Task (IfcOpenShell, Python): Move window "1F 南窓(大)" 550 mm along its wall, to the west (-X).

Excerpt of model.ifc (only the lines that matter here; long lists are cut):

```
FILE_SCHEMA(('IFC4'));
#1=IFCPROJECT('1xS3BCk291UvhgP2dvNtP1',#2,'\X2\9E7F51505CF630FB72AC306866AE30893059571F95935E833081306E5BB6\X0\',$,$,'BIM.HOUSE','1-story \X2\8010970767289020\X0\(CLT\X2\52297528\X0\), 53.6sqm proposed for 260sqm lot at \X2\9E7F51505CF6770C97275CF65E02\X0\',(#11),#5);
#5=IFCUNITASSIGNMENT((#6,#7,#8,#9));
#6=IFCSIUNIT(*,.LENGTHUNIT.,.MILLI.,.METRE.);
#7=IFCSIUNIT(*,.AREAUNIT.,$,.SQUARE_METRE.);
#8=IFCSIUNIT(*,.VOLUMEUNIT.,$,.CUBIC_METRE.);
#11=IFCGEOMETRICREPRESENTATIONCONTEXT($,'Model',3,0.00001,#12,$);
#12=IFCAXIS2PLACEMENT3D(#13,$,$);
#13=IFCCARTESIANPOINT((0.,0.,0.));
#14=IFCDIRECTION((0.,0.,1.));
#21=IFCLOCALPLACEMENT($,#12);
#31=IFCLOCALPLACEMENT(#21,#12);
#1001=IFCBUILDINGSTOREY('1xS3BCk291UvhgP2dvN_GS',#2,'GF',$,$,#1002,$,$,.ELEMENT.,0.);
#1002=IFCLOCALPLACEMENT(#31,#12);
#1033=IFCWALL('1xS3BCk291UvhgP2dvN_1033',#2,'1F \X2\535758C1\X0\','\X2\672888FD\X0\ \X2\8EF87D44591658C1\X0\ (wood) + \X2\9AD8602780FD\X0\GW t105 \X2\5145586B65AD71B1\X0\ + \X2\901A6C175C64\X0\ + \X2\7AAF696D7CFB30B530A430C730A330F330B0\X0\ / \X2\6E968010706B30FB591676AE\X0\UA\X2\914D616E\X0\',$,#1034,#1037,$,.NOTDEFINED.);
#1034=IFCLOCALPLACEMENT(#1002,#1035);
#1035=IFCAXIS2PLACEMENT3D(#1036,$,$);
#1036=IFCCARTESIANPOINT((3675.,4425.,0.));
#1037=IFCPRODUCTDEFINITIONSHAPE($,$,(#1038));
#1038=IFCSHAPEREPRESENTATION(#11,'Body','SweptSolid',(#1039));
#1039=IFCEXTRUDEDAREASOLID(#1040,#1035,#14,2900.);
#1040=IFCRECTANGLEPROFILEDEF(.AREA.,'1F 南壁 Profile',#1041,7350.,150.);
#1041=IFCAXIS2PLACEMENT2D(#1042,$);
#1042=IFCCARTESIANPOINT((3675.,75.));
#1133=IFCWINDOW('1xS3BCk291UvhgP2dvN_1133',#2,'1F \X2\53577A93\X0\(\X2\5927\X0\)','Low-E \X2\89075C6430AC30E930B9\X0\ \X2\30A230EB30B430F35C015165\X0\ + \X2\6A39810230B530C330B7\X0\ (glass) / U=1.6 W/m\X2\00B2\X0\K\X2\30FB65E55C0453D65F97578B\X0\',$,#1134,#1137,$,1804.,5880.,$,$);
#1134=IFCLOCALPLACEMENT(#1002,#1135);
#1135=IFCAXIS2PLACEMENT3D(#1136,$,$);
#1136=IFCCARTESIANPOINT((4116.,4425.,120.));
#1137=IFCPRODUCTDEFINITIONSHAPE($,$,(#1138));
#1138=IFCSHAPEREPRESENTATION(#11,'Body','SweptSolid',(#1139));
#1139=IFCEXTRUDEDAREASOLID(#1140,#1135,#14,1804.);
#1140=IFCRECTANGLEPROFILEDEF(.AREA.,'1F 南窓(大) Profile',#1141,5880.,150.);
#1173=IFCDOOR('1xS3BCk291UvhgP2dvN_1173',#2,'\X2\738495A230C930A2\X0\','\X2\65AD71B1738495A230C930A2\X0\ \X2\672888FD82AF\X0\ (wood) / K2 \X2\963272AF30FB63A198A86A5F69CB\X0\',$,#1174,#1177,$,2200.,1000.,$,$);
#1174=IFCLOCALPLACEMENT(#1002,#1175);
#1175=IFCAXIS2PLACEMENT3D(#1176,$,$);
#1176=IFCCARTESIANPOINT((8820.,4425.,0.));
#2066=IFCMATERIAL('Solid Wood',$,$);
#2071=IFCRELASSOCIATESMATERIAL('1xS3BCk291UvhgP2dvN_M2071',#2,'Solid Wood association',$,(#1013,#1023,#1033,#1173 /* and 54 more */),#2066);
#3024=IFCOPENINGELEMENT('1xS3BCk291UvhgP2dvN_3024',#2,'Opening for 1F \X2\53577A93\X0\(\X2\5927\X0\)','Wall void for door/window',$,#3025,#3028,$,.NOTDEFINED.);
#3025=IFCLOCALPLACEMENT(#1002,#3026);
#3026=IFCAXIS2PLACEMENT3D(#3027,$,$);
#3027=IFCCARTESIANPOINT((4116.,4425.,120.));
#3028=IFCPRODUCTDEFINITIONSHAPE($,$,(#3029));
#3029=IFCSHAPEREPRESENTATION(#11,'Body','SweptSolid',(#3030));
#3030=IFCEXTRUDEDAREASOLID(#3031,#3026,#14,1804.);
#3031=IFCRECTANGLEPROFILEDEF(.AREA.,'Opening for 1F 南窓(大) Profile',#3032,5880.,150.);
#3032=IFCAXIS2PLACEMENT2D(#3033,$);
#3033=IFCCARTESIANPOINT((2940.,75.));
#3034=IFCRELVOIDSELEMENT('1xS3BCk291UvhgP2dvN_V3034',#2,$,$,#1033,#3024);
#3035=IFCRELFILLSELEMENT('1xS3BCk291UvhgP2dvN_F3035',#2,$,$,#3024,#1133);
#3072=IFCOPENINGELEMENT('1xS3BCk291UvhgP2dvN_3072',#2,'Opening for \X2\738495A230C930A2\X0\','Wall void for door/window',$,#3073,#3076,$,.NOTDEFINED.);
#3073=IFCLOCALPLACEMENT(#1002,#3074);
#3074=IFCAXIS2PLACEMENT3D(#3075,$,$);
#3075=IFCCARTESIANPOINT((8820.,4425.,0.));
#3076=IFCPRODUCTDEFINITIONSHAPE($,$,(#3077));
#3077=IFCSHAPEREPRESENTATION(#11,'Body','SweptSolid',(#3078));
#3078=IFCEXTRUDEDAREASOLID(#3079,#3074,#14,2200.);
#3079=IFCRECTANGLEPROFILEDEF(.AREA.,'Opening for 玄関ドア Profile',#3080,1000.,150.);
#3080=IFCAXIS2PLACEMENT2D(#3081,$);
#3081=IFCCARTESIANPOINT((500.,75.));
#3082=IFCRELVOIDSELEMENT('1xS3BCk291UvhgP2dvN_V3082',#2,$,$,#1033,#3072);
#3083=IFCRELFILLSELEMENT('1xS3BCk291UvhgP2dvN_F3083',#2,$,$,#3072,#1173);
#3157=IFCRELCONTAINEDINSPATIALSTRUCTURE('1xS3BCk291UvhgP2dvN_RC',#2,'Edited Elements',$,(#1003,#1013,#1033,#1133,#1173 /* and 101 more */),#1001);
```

```python
import ifcopenshell
import ifcopenshell.api.geometry
import ifcopenshell.util.placement

model = ifcopenshell.open("model.ifc")

window = model.by_guid("1xS3BCk291UvhgP2dvN_1133")
opening = window.FillsVoids[0].RelatingOpeningElement
wall = opening.VoidsElements[0].RelatingBuildingElement

wall_matrix = ifcopenshell.util.placement.get_local_placement(wall.ObjectPlacement)
shift = wall_matrix[:3, 0] * -550.0
before = ifcopenshell.util.placement.get_local_placement(window.ObjectPlacement)[:3, 3].copy()

# The window is not placed relative to its opening, so move both.
for product in (opening, window):
    matrix = ifcopenshell.util.placement.get_local_placement(product.ObjectPlacement)
    matrix[:3, 3] += shift
    ifcopenshell.api.geometry.edit_object_placement(model, product=product, matrix=matrix, is_si=False)

after = ifcopenshell.util.placement.get_local_placement(window.ObjectPlacement)[:3, 3]
print("window moved by", (after - before).round(3) + 0.0)

model.write("model-out.ifc")
```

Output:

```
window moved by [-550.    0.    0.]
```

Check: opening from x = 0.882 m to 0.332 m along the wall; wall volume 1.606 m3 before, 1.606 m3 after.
